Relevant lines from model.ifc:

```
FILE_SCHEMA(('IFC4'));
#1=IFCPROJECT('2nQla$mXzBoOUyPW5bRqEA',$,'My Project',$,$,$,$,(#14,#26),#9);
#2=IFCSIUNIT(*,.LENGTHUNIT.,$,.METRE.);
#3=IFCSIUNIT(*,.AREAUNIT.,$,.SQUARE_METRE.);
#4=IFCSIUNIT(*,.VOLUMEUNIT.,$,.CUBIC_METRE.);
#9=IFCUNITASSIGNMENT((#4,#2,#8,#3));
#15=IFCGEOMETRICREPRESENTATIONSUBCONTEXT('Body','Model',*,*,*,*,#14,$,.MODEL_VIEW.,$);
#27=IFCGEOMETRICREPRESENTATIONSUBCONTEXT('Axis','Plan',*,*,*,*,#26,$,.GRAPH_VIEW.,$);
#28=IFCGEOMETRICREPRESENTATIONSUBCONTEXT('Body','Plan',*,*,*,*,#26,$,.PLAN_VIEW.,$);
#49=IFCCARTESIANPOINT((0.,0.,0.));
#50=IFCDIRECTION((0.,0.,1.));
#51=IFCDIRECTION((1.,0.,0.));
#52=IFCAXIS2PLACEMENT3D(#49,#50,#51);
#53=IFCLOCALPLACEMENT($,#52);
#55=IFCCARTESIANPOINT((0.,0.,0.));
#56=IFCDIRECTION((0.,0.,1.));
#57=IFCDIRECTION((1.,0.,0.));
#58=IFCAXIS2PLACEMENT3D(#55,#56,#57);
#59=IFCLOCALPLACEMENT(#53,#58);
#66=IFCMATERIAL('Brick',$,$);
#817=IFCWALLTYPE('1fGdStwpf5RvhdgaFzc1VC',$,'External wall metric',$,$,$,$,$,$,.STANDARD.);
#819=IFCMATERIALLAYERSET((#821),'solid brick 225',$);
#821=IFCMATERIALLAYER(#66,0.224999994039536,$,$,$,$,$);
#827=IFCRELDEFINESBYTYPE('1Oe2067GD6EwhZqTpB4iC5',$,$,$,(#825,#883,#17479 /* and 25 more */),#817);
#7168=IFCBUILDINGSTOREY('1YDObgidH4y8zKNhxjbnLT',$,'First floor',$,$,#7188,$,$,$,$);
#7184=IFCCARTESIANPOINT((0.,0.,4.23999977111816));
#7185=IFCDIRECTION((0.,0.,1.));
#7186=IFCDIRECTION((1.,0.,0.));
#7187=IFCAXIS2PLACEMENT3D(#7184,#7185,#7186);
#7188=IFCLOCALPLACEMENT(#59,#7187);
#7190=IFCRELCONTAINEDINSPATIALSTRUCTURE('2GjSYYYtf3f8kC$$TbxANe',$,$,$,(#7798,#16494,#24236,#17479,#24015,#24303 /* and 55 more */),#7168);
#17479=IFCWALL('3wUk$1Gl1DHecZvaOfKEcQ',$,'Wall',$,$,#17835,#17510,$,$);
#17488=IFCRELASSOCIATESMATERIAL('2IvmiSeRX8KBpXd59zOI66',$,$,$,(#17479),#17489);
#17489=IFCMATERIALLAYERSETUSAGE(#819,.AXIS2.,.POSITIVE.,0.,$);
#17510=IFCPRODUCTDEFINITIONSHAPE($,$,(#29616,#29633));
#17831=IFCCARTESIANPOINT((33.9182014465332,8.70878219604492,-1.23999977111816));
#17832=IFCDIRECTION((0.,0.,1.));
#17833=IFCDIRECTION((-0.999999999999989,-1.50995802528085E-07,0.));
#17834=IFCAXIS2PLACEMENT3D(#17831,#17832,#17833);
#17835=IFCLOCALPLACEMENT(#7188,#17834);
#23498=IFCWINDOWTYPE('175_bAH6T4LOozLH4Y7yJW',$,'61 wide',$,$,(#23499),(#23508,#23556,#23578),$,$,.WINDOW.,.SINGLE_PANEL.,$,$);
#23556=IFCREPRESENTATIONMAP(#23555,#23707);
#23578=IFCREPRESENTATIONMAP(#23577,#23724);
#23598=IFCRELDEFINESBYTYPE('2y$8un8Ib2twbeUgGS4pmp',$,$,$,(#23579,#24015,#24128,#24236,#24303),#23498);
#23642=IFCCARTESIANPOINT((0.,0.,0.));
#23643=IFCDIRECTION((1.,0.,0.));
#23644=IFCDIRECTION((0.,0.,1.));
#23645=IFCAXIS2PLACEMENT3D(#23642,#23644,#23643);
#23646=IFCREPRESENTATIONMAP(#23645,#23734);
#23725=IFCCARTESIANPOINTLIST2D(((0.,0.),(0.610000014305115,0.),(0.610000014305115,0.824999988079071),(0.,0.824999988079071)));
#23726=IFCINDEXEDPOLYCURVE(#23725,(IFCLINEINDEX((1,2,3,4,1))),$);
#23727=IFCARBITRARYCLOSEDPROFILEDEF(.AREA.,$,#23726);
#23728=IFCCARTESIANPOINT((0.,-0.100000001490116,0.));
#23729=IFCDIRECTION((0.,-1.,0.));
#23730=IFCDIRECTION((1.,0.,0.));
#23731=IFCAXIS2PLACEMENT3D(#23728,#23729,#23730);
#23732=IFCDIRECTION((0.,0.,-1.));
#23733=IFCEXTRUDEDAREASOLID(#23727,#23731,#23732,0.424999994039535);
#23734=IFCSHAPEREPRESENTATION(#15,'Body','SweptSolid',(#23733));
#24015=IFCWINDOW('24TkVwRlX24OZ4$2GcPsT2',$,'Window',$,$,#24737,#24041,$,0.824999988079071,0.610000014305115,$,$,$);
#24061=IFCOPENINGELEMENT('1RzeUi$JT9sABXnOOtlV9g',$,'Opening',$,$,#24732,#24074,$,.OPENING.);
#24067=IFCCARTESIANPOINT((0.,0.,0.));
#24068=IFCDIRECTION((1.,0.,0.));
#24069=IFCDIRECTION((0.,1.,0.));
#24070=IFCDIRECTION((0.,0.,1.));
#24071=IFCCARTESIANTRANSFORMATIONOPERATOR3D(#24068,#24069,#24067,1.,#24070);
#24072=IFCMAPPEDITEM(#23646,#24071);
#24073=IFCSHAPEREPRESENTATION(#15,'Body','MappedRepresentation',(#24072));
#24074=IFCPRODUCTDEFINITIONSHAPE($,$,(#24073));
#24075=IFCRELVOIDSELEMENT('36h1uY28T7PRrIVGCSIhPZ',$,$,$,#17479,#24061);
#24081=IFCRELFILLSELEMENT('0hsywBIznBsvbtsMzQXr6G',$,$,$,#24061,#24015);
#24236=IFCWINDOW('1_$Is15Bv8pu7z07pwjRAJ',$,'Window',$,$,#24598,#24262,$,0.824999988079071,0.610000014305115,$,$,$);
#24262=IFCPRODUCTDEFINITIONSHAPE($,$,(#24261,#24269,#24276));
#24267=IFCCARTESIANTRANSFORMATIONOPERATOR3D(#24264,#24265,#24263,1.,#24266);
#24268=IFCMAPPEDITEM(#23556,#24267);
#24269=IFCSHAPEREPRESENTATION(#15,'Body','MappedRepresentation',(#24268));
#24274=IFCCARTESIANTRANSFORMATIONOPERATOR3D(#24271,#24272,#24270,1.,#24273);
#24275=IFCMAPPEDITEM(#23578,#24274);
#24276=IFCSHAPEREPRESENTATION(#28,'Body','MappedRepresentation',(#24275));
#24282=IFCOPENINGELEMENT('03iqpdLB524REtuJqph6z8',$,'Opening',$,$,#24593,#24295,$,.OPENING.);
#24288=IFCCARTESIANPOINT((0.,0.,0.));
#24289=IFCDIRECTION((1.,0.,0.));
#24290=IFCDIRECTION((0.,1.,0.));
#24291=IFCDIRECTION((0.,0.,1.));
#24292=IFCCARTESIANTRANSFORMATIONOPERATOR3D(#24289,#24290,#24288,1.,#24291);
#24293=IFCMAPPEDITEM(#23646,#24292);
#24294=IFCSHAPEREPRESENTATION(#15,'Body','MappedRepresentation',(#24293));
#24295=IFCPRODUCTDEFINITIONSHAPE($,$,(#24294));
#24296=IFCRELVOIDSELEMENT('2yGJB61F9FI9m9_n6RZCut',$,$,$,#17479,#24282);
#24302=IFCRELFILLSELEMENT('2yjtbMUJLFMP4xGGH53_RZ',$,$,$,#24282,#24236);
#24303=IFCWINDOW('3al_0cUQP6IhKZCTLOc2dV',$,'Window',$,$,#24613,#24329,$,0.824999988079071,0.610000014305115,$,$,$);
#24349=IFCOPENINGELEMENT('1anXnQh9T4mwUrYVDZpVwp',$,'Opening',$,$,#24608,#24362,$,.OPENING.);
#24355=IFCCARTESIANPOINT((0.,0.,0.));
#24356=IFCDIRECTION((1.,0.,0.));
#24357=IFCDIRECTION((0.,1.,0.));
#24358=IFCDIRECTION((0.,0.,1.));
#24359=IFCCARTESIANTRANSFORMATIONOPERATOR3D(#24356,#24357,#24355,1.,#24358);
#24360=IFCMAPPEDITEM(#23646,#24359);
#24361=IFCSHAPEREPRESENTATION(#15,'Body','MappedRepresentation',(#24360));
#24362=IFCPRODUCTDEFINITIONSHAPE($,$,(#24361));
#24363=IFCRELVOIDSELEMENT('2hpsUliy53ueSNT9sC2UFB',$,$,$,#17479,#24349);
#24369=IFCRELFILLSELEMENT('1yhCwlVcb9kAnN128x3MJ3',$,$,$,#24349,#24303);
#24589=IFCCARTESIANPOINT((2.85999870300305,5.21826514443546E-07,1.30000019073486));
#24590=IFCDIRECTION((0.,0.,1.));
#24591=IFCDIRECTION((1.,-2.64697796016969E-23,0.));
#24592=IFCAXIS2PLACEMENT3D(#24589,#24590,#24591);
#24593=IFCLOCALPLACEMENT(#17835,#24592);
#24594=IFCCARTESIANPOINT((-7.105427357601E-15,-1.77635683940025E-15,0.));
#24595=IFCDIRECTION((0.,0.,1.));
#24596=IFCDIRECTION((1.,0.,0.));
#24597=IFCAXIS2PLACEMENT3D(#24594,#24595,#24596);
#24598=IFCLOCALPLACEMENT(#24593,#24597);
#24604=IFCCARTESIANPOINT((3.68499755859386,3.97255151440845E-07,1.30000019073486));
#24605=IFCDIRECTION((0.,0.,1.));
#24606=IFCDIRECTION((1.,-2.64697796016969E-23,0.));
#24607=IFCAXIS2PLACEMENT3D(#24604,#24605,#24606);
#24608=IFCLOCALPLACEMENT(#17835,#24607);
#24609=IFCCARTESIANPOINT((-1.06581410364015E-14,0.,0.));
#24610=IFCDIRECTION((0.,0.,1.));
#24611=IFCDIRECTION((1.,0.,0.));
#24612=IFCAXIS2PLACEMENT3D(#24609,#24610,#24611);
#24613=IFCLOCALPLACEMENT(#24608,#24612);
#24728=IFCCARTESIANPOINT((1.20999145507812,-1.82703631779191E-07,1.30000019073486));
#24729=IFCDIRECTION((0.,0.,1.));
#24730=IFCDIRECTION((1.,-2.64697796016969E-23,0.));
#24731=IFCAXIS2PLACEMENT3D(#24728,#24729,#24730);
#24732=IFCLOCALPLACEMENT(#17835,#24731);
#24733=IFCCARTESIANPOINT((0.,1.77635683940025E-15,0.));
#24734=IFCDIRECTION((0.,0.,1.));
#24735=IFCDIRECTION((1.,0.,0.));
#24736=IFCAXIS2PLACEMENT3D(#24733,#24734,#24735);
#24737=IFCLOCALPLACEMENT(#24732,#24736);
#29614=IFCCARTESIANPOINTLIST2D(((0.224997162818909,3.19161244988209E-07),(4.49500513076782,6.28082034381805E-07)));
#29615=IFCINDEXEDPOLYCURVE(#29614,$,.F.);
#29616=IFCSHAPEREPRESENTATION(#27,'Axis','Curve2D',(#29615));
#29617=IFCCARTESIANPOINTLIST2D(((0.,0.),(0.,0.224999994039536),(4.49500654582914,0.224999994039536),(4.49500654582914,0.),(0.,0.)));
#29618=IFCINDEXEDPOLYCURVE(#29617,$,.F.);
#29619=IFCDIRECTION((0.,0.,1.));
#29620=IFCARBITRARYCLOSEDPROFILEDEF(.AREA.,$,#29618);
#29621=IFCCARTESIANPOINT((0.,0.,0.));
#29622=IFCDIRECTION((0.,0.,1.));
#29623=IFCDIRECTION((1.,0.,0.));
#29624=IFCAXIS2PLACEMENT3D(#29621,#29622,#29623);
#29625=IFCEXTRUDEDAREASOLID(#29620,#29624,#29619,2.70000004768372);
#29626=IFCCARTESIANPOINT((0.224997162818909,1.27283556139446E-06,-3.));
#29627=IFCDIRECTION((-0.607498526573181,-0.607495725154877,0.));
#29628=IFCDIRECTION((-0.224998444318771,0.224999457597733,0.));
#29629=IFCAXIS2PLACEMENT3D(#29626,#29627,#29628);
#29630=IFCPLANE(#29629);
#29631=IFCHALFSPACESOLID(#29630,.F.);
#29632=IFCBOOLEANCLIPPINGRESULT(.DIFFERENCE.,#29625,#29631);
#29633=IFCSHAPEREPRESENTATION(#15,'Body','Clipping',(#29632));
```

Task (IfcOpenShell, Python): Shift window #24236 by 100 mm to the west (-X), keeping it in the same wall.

```python
import ifcopenshell
import ifcopenshell.api.geometry
import ifcopenshell.util.placement
import ifcopenshell.util.unit

model = ifcopenshell.open("model.ifc")
unit_scale = ifcopenshell.util.unit.calculate_unit_scale(model)

window = model.by_guid("1_$Is15Bv8pu7z07pwjRAJ")
opening = window.FillsVoids[0].RelatingOpeningElement
wall = opening.VoidsElements[0].RelatingBuildingElement

wall_matrix = ifcopenshell.util.placement.get_local_placement(wall.ObjectPlacement)
shift = wall_matrix[:3, 0] * 0.1 / unit_scale
before = ifcopenshell.util.placement.get_local_placement(window.ObjectPlacement)[:3, 3].copy()

# The window is placed relative to its opening, so it follows when the opening moves.
matrix = ifcopenshell.util.placement.get_local_placement(opening.ObjectPlacement)
matrix[:3, 3] += shift
ifcopenshell.api.geometry.edit_object_placement(
    model, product=opening, matrix=matrix, is_si=False, should_transform_children=True
)

after = ifcopenshell.util.placement.get_local_placement(window.ObjectPlacement)[:3, 3]
print("window moved by", (after - before).round(3) + 0.0)

model.write("model_edited.ifc")
```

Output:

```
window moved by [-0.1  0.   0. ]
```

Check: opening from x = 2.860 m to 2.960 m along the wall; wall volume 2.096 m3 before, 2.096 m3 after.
